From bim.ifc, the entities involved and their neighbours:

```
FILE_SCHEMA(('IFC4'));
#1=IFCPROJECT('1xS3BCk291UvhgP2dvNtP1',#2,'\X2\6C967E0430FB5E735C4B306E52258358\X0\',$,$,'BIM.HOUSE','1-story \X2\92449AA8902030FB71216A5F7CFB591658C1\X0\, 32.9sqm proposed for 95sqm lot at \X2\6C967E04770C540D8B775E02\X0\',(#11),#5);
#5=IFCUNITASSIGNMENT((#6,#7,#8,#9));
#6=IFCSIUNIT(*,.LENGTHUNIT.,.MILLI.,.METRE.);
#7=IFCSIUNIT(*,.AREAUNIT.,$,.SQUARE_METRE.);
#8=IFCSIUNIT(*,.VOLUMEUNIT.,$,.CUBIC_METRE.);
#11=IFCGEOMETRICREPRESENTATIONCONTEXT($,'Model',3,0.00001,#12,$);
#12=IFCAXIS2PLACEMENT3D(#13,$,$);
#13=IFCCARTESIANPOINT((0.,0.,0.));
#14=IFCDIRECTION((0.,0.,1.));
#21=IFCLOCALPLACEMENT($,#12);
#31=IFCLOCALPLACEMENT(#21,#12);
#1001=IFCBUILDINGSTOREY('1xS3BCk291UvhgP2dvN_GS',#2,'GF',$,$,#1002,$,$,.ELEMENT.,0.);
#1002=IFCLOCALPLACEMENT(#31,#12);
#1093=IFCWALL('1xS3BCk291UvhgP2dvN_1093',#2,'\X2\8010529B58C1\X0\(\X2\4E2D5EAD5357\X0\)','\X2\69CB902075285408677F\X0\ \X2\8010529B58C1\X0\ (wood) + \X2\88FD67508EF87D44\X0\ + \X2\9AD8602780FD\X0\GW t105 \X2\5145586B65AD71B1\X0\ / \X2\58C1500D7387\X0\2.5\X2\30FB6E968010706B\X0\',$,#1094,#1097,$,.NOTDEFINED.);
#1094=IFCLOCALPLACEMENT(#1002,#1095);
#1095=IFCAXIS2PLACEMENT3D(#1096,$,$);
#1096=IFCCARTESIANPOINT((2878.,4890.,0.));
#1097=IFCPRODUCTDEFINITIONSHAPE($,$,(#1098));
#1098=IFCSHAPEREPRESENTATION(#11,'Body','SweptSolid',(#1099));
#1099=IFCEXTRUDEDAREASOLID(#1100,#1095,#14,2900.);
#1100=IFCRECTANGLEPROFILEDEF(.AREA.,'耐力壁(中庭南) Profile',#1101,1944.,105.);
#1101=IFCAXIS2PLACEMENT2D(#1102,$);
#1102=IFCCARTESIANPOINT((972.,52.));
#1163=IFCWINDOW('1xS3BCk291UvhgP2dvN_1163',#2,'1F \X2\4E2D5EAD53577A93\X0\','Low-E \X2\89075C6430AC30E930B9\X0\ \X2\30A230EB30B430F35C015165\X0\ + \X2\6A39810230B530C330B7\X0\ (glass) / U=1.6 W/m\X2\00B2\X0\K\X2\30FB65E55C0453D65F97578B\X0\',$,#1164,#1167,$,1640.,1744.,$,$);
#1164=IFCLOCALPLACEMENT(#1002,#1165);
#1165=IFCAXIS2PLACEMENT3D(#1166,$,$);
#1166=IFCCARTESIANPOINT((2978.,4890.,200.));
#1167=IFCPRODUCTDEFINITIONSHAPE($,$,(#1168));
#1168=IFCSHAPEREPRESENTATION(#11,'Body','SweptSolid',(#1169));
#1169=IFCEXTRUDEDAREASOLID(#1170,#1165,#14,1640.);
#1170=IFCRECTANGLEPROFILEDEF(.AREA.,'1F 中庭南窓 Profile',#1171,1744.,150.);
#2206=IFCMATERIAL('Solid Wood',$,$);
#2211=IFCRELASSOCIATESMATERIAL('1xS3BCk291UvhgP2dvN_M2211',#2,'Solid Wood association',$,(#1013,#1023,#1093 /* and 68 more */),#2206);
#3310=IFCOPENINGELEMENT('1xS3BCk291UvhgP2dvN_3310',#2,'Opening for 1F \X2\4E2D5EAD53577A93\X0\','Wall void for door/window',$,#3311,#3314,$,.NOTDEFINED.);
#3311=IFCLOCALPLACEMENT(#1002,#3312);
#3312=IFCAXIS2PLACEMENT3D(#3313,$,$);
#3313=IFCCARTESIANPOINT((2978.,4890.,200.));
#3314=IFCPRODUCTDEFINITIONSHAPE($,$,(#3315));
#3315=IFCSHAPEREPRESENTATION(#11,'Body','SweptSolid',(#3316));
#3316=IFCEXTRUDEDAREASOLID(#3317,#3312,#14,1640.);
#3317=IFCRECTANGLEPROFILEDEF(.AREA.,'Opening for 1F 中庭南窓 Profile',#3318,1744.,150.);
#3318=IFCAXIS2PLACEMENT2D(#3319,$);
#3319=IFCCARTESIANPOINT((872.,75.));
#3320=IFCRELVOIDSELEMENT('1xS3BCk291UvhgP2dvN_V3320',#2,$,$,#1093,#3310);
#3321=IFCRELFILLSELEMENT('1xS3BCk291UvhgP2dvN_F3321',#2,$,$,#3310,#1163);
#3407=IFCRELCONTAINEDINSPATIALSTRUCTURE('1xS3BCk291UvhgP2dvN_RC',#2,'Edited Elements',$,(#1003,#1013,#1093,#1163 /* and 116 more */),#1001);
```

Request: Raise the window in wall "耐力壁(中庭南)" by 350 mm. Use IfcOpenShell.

```python
import numpy as np
import ifcopenshell
import ifcopenshell.api.geometry
import ifcopenshell.util.placement
import ifcopenshell.util.unit

model = ifcopenshell.open("bim.ifc")
unit_scale = ifcopenshell.util.unit.calculate_unit_scale(model)

window = model.by_id(1163)
opening = window.FillsVoids[0].RelatingOpeningElement
dz = 0.35 / unit_scale

shift = np.array([0.0, 0.0, dz])
# The window is not placed relative to its opening, so move both.
for product in (opening, window):
    matrix = ifcopenshell.util.placement.get_local_placement(product.ObjectPlacement)
    matrix[:3, 3] += shift
    ifcopenshell.api.geometry.edit_object_placement(model, product=product, matrix=matrix, is_si=False)

print(f"moved by {dz * unit_scale:+.3f} m")

model.write("bim_updated.ifc")
```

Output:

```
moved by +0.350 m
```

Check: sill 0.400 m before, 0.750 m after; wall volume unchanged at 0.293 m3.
